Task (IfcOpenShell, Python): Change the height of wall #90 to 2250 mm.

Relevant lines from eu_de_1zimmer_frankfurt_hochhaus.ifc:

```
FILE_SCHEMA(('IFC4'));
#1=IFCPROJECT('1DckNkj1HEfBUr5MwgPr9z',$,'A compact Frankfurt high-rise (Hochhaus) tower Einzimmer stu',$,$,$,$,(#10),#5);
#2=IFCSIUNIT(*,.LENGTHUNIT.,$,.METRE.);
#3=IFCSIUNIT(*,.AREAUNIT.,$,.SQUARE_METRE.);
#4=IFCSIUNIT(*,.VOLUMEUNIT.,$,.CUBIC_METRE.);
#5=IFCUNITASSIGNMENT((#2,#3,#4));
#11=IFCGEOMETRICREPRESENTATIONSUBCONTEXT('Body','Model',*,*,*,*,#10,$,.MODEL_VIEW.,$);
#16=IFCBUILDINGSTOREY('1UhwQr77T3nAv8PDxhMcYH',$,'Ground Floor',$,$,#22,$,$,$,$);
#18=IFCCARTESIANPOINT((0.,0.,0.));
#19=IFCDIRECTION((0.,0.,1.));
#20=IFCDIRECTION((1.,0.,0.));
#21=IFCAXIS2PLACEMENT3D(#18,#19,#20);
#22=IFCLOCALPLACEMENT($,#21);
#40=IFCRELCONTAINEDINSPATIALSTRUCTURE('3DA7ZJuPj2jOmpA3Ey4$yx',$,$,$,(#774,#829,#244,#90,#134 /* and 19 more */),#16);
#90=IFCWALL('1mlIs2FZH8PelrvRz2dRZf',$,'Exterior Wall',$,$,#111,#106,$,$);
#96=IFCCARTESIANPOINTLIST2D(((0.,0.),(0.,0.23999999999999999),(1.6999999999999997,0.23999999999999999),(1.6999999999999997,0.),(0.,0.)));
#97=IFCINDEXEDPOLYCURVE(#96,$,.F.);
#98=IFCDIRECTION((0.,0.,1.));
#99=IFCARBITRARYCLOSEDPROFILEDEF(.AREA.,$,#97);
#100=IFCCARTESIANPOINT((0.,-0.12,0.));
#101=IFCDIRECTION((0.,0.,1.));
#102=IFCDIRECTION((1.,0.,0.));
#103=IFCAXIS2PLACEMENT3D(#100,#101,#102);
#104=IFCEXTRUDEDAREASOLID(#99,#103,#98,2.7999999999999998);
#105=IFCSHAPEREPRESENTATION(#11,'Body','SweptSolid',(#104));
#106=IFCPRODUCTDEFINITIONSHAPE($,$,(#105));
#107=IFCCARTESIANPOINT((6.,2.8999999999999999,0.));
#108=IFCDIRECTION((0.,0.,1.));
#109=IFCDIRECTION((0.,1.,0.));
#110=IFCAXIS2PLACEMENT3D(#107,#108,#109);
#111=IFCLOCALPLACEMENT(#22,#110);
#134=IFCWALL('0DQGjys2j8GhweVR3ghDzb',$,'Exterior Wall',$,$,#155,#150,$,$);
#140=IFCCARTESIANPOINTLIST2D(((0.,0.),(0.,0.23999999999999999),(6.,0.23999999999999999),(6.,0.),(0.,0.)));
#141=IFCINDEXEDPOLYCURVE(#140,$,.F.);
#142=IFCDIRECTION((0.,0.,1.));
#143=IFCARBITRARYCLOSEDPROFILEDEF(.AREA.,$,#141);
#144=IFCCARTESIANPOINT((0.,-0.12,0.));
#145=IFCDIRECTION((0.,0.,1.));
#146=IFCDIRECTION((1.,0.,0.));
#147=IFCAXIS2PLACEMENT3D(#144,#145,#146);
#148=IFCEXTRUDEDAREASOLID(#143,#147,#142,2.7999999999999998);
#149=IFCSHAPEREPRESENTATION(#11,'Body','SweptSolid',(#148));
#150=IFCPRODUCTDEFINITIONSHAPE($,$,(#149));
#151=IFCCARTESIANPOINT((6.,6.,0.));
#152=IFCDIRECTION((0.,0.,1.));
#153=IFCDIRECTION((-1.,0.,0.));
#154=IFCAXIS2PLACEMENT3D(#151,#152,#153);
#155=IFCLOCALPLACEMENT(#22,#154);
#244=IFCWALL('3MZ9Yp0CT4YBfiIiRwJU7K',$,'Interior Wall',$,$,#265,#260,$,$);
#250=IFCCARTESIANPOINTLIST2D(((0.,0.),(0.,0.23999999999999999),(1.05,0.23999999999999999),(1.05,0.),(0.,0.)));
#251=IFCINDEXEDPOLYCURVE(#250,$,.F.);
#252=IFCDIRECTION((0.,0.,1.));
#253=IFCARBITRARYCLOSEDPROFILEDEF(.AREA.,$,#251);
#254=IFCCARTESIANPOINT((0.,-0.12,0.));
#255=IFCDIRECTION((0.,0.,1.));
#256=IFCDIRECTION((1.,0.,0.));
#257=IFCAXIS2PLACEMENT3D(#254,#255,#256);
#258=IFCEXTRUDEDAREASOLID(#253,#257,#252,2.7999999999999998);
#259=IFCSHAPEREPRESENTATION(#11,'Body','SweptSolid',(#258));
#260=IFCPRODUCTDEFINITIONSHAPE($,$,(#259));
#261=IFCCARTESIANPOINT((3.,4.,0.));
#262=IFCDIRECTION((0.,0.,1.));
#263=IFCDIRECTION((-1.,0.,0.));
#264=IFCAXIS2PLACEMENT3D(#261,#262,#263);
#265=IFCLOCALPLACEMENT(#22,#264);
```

```python
import ifcopenshell
import ifcopenshell.geom
import ifcopenshell.util.representation
import ifcopenshell.util.shape
import ifcopenshell.util.unit

model = ifcopenshell.open("eu_de_1zimmer_frankfurt_hochhaus.ifc")
unit_scale = ifcopenshell.util.unit.calculate_unit_scale(model)
settings = ifcopenshell.geom.settings()


def volume(element):
    """Net volume in cubic metres, openings subtracted."""
    shape = ifcopenshell.geom.create_shape(settings, element)
    return ifcopenshell.util.shape.get_volume(shape.geometry)


wall = model.by_guid("1mlIs2FZH8PelrvRz2dRZf")
before = volume(wall)

body = ifcopenshell.util.representation.get_representation(wall, "Model", "Body")
solid = body.Items[0]
old_height = solid.Depth
solid.Depth = 2.25 / unit_scale
after = volume(wall)

print(f"height {old_height:g} -> {solid.Depth:g}, volume {before:.3f} -> {after:.3f} m3")

model.write("eu_de_1zimmer_frankfurt_hochhaus_edited.ifc")
```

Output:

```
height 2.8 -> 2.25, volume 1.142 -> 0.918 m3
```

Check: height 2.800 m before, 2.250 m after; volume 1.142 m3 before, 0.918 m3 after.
